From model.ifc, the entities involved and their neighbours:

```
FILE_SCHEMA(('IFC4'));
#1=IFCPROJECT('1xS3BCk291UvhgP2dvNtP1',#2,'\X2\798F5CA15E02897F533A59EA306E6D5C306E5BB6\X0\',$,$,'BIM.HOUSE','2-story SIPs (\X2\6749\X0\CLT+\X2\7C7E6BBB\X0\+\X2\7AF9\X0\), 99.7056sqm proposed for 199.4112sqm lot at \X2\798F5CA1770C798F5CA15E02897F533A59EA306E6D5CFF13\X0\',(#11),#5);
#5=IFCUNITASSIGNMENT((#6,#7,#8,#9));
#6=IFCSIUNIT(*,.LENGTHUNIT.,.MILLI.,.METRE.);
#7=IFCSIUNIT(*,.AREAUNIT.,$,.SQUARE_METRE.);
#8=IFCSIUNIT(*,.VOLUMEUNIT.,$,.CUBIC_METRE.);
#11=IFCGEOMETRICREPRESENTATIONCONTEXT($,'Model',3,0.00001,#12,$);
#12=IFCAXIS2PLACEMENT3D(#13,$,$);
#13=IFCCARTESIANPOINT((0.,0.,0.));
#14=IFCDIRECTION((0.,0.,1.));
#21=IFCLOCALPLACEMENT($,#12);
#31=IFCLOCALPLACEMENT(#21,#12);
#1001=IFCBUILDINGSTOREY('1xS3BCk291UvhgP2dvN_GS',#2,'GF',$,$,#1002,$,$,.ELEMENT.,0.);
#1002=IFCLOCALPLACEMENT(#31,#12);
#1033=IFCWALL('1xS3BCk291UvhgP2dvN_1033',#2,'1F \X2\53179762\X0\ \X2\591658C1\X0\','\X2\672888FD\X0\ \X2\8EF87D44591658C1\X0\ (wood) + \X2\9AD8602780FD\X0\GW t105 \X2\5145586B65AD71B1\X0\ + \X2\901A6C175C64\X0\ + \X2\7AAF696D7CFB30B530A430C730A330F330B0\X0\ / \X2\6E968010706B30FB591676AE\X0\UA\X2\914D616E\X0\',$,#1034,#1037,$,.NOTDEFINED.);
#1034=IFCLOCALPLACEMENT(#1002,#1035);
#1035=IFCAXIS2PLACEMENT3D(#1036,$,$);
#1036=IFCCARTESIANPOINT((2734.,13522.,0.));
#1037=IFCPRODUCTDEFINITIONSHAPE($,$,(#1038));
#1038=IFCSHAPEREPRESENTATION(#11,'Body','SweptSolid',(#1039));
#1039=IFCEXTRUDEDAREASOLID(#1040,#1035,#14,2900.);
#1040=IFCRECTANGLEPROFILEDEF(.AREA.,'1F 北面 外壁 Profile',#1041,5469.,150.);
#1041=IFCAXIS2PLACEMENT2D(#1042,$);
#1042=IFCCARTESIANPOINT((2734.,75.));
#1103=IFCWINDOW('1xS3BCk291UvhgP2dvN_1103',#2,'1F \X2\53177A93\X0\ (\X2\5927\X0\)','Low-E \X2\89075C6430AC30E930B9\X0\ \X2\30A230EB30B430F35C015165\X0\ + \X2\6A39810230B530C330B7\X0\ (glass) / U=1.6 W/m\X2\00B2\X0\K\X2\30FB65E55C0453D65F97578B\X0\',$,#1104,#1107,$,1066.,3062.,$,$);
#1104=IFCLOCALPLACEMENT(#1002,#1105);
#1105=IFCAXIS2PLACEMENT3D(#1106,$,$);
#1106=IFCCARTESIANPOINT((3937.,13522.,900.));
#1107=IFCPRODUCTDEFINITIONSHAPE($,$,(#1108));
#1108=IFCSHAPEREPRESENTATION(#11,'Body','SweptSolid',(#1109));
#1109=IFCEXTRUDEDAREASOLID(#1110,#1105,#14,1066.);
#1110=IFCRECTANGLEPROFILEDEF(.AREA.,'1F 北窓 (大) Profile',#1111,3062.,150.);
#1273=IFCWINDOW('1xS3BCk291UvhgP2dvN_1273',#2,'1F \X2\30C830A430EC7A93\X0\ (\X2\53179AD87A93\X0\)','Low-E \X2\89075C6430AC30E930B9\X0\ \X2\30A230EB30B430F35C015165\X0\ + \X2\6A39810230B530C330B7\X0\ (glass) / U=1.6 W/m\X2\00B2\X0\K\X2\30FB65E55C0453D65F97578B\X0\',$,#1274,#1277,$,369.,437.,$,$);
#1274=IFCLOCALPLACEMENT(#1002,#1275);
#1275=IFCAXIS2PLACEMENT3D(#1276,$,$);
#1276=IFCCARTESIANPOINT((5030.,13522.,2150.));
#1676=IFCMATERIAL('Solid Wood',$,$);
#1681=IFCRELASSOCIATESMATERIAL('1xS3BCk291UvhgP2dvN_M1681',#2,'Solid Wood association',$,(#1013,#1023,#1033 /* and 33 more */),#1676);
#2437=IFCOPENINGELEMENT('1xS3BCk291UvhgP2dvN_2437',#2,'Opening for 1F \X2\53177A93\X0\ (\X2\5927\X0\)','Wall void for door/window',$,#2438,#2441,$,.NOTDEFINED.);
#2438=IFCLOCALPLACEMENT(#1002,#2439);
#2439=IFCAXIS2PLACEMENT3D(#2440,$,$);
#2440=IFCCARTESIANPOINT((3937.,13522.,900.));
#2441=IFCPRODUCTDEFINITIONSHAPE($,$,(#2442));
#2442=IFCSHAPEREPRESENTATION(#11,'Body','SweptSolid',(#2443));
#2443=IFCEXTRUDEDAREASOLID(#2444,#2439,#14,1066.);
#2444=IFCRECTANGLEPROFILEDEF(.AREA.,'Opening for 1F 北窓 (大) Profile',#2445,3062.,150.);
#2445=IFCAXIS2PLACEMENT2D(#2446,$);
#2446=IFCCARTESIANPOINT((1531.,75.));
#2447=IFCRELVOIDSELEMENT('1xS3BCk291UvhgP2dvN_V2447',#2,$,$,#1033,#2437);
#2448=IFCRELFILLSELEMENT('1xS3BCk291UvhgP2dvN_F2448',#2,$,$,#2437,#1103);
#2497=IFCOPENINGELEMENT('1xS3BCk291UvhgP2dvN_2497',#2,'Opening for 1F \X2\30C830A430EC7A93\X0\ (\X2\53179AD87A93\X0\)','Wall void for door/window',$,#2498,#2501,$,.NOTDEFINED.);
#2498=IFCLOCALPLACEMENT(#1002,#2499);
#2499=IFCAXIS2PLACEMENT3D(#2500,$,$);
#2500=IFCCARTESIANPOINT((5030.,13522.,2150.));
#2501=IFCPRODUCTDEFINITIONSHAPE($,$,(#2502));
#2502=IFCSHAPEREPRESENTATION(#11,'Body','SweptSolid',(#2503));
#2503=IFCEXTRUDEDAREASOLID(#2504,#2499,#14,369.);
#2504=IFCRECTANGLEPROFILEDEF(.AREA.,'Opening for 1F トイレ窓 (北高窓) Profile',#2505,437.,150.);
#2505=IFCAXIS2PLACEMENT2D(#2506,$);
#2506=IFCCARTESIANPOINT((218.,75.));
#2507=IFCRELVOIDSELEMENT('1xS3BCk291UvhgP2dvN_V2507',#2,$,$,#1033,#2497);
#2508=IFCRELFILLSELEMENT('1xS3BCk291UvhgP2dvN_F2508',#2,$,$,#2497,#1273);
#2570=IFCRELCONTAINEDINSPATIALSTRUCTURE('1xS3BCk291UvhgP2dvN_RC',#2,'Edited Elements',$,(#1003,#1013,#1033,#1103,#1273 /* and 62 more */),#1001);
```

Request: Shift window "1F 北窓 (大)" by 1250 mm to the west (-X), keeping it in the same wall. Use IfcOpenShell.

```python
import ifcopenshell
import ifcopenshell.api.geometry
import ifcopenshell.util.placement

model = ifcopenshell.open("model.ifc")

window = model.by_id(1103)
opening = window.FillsVoids[0].RelatingOpeningElement
wall = opening.VoidsElements[0].RelatingBuildingElement

wall_matrix = ifcopenshell.util.placement.get_local_placement(wall.ObjectPlacement)
shift = wall_matrix[:3, 0] * -1250.0
before = ifcopenshell.util.placement.get_local_placement(window.ObjectPlacement)[:3, 3].copy()

# The window is not placed relative to its opening, so move both.
for product in (opening, window):
    matrix = ifcopenshell.util.placement.get_local_placement(product.ObjectPlacement)
    matrix[:3, 3] += shift
    ifcopenshell.api.geometry.edit_object_placement(model, product=product, matrix=matrix, is_si=False)

after = ifcopenshell.util.placement.get_local_placement(window.ObjectPlacement)[:3, 3]
print("window moved by", (after - before).round(3) + 0.0)

model.write("model_v2.ifc")
```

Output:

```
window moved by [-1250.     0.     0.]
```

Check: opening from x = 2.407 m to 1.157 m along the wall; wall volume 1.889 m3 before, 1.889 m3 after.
